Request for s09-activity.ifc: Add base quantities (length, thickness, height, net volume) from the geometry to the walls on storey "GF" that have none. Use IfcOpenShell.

First a look at what the model holds.

```python
import ifcopenshell
import ifcopenshell.util.element
import ifcopenshell.util.unit

model = ifcopenshell.open("s09-activity.ifc")
print(model.schema)
for unit_type in ("LENGTHUNIT", "AREAUNIT", "VOLUMEUNIT"):
    print(unit_type, ifcopenshell.util.unit.calculate_unit_scale(model, unit_type))
storey = next(s for s in model.by_type("IfcBuildingStorey") if s.Name == "GF")
walls = [e for e in ifcopenshell.util.element.get_decomposition(storey) if e.is_a("IfcWall")]
for e in sorted(walls, key=lambda e: e.id()):
    print(e.id(), e.is_a(), e.Name, list(ifcopenshell.util.element.get_psets(e, qtos_only=True)), sep=" | ")
```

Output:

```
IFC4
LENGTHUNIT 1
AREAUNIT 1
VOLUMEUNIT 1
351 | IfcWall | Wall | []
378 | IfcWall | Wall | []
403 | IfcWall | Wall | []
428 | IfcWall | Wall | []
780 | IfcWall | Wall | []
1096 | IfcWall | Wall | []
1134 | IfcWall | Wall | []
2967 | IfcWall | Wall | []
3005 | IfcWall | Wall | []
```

```python
import ifcopenshell
import ifcopenshell.api.pset
import ifcopenshell.geom
import ifcopenshell.util.element
import ifcopenshell.util.shape
import ifcopenshell.util.unit

model = ifcopenshell.open("s09-activity.ifc")
unit_scale = ifcopenshell.util.unit.calculate_unit_scale(model)
volume_scale = ifcopenshell.util.unit.calculate_unit_scale(model, "VOLUMEUNIT")
settings = ifcopenshell.geom.settings()

storey = next(s for s in model.by_type("IfcBuildingStorey") if s.Name == "GF")
walls = [e for e in ifcopenshell.util.element.get_decomposition(storey) if e.is_a("IfcWall")]

for e in sorted(walls, key=lambda e: e.id()):
    if ifcopenshell.util.element.get_psets(e, qtos_only=True, should_inherit=False):
        continue
    # Geometry comes back in metres, in the element's own axes.
    shape = ifcopenshell.geom.create_shape(settings, e)
    values = {
        "Length": ifcopenshell.util.shape.get_x(shape.geometry) / unit_scale,
        "Width": ifcopenshell.util.shape.get_y(shape.geometry) / unit_scale,
        "Height": ifcopenshell.util.shape.get_z(shape.geometry) / unit_scale,
        "NetVolume": ifcopenshell.util.shape.get_volume(shape.geometry) / volume_scale,
    }
    qto = ifcopenshell.api.pset.add_qto(model, product=e, name="Qto_WallBaseQuantities")
    ifcopenshell.api.pset.edit_qto(model, qto=qto, properties=values)
    print(e.id(), {k: round(v, 3) for k, v in values.items()})

model.write("s09-activity_rev.ifc")
```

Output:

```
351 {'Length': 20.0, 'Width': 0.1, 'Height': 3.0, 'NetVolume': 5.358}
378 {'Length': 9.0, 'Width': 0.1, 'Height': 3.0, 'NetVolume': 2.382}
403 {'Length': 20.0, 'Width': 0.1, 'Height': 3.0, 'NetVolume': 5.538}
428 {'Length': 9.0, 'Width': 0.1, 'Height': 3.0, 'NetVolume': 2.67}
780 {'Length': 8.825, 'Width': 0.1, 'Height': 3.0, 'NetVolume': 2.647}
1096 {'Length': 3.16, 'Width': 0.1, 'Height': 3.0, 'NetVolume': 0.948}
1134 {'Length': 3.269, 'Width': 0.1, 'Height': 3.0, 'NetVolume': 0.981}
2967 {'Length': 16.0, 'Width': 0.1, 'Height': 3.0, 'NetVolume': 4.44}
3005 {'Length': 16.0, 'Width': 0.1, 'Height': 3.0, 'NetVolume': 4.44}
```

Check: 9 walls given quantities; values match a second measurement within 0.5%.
